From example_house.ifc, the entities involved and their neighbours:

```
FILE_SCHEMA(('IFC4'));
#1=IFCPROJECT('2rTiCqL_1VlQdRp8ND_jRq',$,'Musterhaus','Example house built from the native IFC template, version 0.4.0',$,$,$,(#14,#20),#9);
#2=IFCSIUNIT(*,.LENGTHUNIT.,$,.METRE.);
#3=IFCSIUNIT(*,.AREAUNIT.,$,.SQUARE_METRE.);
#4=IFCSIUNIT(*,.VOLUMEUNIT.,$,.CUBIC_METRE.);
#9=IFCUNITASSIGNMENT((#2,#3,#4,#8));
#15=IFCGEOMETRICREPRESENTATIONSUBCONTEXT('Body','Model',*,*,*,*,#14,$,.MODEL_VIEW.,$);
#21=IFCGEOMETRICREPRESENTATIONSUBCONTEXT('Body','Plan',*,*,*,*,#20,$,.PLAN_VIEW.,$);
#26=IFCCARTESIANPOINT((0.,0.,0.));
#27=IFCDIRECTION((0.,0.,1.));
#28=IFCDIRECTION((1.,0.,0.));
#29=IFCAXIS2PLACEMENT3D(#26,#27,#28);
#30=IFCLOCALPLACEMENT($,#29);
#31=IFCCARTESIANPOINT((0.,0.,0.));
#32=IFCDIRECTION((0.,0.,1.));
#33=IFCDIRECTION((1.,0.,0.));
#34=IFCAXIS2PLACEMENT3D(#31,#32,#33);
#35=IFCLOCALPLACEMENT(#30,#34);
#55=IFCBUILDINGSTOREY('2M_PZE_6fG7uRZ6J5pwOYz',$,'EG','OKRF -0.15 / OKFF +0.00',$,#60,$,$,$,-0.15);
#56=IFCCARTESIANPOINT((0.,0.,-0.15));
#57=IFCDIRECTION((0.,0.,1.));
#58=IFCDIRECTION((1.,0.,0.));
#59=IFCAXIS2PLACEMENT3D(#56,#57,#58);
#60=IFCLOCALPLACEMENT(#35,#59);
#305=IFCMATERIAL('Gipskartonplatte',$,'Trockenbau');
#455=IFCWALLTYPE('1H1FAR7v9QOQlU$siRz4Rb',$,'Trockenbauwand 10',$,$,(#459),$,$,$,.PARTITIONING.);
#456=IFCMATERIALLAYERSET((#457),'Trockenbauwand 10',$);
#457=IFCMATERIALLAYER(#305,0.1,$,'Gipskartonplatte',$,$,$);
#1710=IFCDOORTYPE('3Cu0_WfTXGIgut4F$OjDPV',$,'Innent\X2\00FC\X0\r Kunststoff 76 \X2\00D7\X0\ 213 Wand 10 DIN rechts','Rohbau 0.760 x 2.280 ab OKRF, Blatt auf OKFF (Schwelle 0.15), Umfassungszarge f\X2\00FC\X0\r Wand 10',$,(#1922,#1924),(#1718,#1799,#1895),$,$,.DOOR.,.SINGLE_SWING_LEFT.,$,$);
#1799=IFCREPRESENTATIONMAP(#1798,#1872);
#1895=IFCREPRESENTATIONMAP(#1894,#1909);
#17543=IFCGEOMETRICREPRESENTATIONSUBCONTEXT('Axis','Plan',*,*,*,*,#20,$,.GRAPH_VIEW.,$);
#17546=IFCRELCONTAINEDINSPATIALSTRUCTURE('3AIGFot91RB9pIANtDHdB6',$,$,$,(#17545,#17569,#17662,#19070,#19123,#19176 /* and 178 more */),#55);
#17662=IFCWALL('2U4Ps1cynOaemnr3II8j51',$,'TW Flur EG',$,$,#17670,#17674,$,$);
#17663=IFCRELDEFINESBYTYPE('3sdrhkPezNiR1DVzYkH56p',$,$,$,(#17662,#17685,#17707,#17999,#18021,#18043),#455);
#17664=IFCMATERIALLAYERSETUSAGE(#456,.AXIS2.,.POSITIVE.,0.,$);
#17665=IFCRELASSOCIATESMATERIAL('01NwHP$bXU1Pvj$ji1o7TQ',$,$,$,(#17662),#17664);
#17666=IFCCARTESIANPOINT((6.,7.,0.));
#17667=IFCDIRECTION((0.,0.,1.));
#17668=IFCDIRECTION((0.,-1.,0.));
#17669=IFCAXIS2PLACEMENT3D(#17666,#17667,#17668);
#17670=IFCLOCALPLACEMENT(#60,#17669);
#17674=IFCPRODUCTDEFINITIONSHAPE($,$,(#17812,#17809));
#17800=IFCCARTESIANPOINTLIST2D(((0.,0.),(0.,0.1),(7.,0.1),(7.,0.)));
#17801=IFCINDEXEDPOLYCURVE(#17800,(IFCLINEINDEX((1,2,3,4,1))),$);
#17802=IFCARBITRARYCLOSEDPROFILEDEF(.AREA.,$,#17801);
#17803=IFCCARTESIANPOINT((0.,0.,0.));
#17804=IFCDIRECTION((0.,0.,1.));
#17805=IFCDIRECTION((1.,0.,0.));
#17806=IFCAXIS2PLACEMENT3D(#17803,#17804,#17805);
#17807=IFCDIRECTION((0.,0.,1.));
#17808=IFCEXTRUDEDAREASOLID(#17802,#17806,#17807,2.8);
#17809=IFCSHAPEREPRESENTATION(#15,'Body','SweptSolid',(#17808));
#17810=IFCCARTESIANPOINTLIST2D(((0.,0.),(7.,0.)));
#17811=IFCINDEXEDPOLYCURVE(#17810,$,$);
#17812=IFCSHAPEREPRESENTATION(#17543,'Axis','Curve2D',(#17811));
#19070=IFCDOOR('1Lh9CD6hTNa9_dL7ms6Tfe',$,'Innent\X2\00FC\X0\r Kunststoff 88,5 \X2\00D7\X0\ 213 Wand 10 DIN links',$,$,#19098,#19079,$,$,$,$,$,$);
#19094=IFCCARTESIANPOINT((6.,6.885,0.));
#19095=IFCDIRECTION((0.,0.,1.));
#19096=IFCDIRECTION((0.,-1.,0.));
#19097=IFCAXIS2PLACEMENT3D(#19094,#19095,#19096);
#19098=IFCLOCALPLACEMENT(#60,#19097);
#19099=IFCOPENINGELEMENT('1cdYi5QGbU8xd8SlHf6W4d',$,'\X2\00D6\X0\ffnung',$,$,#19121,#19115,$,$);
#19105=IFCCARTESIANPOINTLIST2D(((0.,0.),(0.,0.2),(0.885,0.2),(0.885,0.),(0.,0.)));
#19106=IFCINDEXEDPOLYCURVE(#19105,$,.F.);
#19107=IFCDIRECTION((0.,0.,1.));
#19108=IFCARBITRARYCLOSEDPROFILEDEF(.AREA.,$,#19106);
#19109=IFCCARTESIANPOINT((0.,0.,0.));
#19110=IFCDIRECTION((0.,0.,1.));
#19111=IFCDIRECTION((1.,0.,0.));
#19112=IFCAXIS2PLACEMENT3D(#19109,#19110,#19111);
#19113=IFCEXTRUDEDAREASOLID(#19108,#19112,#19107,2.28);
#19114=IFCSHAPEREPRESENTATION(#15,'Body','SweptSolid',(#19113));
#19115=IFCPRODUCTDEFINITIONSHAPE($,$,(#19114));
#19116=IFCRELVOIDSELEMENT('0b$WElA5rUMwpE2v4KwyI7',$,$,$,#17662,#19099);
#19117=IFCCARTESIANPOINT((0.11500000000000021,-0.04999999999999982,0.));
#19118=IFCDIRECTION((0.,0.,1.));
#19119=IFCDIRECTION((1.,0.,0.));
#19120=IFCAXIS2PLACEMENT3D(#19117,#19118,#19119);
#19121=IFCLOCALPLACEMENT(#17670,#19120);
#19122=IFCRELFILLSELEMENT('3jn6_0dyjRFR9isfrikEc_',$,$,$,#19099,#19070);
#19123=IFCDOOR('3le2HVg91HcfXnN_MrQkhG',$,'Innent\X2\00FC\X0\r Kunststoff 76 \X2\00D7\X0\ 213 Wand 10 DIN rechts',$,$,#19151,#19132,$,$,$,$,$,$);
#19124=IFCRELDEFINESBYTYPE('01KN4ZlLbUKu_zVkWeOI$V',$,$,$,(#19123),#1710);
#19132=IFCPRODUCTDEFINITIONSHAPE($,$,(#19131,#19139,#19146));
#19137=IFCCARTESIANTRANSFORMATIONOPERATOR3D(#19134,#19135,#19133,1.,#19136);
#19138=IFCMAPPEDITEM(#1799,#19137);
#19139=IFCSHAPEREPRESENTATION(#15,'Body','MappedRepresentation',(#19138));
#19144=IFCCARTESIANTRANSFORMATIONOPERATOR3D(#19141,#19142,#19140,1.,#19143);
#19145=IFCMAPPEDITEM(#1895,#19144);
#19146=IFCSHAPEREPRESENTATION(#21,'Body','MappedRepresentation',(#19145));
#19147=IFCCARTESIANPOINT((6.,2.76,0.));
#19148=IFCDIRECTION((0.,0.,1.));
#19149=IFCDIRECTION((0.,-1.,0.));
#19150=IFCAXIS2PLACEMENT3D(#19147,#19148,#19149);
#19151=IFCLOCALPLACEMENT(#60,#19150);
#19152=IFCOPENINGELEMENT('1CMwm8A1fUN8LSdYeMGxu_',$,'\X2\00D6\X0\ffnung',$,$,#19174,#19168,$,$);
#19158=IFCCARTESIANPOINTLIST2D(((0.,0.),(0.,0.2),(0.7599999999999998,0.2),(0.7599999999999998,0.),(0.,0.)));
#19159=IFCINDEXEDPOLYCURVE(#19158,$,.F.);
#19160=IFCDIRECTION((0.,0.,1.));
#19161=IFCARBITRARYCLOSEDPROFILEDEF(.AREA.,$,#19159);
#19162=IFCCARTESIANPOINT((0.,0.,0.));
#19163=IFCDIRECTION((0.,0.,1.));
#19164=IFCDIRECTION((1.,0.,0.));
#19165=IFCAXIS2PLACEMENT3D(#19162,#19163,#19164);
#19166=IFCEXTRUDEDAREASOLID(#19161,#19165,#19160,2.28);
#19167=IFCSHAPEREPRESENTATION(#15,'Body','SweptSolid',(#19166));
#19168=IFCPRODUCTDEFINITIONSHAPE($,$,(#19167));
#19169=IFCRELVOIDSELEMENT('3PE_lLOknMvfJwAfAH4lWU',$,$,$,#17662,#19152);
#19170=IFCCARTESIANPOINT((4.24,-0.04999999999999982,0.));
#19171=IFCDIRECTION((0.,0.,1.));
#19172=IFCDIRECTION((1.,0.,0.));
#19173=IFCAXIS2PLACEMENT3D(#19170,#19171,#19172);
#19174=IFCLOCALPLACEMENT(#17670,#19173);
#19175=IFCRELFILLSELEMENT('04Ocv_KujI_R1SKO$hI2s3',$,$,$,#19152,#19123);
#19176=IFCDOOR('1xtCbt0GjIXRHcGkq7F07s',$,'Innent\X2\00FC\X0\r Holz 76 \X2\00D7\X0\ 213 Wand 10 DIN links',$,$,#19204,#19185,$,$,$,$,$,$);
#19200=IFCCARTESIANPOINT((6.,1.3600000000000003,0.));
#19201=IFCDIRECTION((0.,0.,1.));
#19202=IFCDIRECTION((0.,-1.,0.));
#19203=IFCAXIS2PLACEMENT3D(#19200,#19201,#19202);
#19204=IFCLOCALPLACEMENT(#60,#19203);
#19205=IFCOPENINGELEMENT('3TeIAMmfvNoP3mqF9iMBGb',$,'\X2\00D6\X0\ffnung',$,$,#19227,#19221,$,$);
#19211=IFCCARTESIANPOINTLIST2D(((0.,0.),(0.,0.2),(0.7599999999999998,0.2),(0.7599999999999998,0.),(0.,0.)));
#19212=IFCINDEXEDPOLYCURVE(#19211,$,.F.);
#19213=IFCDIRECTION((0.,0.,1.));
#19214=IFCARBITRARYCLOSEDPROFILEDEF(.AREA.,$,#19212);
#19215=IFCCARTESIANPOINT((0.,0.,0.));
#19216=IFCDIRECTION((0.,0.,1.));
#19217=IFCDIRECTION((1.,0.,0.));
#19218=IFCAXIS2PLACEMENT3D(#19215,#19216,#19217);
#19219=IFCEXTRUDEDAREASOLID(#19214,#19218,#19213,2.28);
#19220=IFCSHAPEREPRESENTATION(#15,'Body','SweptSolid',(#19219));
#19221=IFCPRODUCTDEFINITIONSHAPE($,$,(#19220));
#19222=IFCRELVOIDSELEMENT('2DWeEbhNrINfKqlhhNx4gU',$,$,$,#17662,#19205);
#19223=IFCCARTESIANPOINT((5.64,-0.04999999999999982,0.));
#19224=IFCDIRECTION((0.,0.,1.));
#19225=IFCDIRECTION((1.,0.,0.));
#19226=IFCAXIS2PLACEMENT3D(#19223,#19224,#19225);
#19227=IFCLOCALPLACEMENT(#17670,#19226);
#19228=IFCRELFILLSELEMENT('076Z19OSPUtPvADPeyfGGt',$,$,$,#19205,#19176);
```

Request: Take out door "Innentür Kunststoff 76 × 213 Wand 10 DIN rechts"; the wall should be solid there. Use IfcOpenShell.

```python
import ifcopenshell
import ifcopenshell.api.feature
import ifcopenshell.api.root
import ifcopenshell.geom
import ifcopenshell.util.shape

model = ifcopenshell.open("example_house.ifc")
settings = ifcopenshell.geom.settings()


def volume(element):
    """Net volume in cubic metres, openings subtracted."""
    shape = ifcopenshell.geom.create_shape(settings, element)
    return ifcopenshell.util.shape.get_volume(shape.geometry)


door = model.by_id(19123)
opening = door.FillsVoids[0].RelatingOpeningElement
wall = opening.VoidsElements[0].RelatingBuildingElement
before = volume(wall)

ifcopenshell.api.root.remove_product(model, product=door)
ifcopenshell.api.feature.remove_feature(model, feature=opening)

after = volume(wall)

print(f"wall volume {before:.3f} -> {after:.3f} m3")

model.write("example_house-out.ifc")
```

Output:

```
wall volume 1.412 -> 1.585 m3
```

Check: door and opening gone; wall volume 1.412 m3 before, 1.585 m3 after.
